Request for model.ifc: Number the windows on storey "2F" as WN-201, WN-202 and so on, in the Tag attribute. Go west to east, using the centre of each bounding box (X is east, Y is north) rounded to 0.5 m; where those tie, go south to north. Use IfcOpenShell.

First a look at what the model holds.

```python
import ifcopenshell
import ifcopenshell.util.element
import ifcopenshell.util.placement

model = ifcopenshell.open("model.ifc")
print(model.schema)
storey = next(s for s in model.by_type("IfcBuildingStorey") if s.Name == "2F")
windows = [e for e in ifcopenshell.util.element.get_decomposition(storey) if e.is_a("IfcWindow")]
for e in sorted(windows, key=lambda e: e.id()):
    origin = ifcopenshell.util.placement.get_local_placement(e.ObjectPlacement)[:3, 3]
    print(e.id(), e.Tag, e.Name, origin.round(2) + 0.0, sep=" | ")
```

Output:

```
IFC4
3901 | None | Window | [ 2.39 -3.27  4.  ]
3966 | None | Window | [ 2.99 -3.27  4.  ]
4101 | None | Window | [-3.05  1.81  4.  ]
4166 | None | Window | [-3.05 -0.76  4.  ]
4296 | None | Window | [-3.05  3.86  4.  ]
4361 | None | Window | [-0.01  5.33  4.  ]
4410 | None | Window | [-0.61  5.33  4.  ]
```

```python
import ifcopenshell
import ifcopenshell.geom
import ifcopenshell.util.element
import ifcopenshell.util.shape

model = ifcopenshell.open("model.ifc")
settings = ifcopenshell.geom.settings()
settings.set("use-world-coords", True)


def centre(element):
    shape = ifcopenshell.geom.create_shape(settings, element)
    return ifcopenshell.util.shape.get_bbox_centroid(shape.geometry)


storey = next(s for s in model.by_type("IfcBuildingStorey") if s.Name == "2F")
windows = [e for e in ifcopenshell.util.element.get_decomposition(storey) if e.is_a("IfcWindow")]

# Insertion points can sit at a corner or the storey origin, so sort by the geometry (in metres).
centres = {e: centre(e) for e in windows}
windows.sort(key=lambda e: (round(centres[e][0] / 0.5), centres[e][1]))

for i, e in enumerate(windows, start=1):
    number = f"WN-2{i:02d}"
    e.Tag = number
    print(e.id(), number)

model.write("model-out.ifc")
```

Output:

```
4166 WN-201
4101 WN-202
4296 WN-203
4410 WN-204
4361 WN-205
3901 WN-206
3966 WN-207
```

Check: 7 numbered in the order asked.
